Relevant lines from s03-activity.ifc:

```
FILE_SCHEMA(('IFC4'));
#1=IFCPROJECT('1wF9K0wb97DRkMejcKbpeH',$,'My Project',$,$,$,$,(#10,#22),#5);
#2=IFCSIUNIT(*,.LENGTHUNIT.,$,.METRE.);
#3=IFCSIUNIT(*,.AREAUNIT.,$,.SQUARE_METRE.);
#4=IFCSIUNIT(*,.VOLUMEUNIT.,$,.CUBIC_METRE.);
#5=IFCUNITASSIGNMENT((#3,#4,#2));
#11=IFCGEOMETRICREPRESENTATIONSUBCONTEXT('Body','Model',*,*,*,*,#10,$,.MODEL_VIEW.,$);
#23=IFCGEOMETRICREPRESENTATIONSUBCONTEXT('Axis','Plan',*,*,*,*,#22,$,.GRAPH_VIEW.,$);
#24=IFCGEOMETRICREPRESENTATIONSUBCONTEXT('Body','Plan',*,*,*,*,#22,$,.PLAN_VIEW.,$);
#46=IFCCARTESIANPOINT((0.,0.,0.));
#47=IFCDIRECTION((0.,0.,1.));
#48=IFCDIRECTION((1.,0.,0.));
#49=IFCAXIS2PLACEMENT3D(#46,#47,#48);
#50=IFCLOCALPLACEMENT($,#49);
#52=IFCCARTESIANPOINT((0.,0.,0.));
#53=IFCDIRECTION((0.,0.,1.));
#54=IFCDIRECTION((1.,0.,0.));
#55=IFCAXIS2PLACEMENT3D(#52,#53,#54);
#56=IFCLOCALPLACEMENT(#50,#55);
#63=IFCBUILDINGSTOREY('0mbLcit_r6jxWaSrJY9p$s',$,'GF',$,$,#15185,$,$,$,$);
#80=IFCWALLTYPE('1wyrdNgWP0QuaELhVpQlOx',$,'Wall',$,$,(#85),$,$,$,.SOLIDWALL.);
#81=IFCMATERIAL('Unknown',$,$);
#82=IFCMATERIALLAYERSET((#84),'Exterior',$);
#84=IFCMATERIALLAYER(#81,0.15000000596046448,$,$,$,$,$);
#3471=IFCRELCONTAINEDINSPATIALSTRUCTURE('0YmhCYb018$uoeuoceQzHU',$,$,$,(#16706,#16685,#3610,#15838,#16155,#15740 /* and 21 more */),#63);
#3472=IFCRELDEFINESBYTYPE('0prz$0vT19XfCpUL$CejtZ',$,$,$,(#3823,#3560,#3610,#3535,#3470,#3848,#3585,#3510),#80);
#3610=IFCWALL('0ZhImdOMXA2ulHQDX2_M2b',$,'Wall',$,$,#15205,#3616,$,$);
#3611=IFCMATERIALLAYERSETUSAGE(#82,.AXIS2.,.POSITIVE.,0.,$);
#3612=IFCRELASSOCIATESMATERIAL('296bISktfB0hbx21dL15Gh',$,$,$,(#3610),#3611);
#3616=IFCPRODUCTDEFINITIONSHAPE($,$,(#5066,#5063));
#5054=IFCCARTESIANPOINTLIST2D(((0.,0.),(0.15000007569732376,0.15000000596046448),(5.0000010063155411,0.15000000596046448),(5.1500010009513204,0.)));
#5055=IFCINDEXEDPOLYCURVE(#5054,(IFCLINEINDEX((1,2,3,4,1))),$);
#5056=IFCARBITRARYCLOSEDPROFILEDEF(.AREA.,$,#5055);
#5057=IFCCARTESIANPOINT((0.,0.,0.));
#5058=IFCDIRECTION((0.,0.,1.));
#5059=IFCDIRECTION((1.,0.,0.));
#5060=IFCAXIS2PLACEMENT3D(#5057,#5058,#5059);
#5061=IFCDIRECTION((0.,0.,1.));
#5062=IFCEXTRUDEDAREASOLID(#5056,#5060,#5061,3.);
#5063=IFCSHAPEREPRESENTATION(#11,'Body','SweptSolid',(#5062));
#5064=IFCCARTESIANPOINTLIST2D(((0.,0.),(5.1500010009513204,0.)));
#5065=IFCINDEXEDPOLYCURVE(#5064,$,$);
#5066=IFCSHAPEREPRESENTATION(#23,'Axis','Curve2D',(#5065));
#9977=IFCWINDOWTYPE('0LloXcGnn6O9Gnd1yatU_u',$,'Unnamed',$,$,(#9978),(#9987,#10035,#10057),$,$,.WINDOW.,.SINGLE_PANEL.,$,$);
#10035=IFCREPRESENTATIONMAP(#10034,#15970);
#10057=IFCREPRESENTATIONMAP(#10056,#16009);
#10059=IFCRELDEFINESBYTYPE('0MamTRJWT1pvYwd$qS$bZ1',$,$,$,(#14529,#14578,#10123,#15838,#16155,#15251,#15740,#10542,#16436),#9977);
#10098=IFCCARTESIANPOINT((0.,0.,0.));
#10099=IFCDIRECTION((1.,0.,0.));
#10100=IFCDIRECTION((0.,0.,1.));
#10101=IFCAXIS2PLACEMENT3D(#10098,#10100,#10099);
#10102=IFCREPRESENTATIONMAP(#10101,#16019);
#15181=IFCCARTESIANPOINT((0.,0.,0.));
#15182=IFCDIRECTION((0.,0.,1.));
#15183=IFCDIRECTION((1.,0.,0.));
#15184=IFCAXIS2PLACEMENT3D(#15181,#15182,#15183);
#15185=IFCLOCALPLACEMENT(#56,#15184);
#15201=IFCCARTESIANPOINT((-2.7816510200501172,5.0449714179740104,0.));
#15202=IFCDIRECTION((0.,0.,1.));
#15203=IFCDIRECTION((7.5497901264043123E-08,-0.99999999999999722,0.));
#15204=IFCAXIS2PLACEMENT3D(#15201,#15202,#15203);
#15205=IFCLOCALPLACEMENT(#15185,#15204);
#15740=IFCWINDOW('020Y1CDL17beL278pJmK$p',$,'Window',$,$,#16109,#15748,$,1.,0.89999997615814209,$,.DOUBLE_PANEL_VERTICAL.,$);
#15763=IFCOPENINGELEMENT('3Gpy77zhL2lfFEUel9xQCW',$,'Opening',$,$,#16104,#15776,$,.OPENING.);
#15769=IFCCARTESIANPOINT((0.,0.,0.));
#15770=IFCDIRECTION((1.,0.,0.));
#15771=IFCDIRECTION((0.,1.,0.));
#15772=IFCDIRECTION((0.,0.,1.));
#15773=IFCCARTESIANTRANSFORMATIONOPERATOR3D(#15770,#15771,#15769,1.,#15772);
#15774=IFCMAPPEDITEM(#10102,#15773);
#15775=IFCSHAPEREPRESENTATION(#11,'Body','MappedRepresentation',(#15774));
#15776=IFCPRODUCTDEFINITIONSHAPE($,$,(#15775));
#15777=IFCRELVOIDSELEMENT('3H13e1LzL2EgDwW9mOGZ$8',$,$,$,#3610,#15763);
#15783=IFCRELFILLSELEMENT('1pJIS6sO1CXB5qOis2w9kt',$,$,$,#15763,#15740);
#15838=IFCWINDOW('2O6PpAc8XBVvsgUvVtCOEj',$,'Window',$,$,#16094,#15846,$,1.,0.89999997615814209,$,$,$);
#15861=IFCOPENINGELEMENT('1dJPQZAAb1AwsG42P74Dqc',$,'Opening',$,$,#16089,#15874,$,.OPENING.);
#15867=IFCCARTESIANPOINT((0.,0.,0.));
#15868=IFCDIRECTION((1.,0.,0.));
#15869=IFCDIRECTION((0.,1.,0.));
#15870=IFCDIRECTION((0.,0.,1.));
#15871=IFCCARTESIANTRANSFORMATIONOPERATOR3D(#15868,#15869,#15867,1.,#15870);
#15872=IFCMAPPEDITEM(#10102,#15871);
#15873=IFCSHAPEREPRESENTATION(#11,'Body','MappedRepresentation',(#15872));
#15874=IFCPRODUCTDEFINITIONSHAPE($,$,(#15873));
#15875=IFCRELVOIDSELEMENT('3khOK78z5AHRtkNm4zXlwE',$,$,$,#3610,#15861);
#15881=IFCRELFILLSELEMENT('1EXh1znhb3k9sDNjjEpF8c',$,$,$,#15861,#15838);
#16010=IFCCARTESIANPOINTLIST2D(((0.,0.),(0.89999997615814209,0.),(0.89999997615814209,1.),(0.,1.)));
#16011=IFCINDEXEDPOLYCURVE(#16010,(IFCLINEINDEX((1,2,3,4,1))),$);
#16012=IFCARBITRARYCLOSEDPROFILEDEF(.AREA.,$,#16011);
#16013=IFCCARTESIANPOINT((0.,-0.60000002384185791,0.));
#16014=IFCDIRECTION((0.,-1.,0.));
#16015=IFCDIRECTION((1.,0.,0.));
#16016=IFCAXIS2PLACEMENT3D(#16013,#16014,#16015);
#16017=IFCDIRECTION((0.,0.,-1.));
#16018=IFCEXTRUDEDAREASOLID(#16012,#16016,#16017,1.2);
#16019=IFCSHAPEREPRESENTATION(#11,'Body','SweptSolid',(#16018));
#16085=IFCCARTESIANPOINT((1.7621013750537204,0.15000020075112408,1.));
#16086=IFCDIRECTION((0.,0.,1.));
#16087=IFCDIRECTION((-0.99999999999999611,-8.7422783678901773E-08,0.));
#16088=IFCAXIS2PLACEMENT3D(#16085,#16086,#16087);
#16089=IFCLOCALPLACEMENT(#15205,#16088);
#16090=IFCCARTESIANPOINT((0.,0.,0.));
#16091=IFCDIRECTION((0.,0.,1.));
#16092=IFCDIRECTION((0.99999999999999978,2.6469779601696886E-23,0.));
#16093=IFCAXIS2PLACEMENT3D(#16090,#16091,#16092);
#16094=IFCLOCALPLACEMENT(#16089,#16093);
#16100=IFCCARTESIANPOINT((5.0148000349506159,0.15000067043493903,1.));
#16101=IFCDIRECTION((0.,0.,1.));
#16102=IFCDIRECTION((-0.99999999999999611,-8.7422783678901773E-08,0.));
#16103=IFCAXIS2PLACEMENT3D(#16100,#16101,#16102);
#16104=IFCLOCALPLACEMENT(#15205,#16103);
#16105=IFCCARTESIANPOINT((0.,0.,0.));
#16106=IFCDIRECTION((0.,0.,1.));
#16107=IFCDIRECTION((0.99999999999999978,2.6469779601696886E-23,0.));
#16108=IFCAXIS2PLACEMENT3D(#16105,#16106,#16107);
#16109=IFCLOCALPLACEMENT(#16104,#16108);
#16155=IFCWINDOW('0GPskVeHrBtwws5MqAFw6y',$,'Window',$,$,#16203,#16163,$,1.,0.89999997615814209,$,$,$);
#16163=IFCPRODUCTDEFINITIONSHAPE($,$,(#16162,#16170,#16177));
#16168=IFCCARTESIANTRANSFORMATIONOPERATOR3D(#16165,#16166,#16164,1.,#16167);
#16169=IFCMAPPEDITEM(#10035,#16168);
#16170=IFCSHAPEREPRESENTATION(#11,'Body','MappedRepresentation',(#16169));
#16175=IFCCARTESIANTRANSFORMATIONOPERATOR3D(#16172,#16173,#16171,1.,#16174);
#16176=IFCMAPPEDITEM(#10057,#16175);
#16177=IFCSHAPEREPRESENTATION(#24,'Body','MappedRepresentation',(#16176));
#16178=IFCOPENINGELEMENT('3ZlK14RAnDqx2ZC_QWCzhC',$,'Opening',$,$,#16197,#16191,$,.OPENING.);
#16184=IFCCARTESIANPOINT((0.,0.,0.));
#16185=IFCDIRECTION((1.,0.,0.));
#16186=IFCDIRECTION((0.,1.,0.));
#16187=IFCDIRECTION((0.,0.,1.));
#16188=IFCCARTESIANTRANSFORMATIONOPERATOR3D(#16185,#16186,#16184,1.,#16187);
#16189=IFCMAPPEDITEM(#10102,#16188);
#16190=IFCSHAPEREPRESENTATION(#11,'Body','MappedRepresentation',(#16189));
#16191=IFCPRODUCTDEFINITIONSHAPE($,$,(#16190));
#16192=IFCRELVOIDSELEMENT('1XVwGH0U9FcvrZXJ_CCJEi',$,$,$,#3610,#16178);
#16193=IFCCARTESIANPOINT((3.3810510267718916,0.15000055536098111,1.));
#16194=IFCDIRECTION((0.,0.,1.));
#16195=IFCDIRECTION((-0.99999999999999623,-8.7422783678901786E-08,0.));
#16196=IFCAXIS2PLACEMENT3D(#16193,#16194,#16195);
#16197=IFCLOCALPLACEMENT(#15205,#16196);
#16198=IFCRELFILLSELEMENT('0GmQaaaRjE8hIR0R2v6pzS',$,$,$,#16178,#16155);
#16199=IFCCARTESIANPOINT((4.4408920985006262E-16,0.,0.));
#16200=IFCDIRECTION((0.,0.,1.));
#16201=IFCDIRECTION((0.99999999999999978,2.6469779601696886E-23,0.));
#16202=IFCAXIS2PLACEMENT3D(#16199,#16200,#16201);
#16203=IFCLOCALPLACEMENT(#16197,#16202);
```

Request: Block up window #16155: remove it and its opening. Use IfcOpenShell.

```python
import ifcopenshell
import ifcopenshell.api.feature
import ifcopenshell.api.root
import ifcopenshell.geom
import ifcopenshell.util.shape

model = ifcopenshell.open("s03-activity.ifc")
settings = ifcopenshell.geom.settings()


def volume(element):
    """Net volume in cubic metres, openings subtracted."""
    shape = ifcopenshell.geom.create_shape(settings, element)
    return ifcopenshell.util.shape.get_volume(shape.geometry)


window = model.by_guid("0GPskVeHrBtwws5MqAFw6y")
opening = window.FillsVoids[0].RelatingOpeningElement
wall = opening.VoidsElements[0].RelatingBuildingElement
before = volume(wall)

ifcopenshell.api.root.remove_product(model, product=window)
ifcopenshell.api.feature.remove_feature(model, feature=opening)

after = volume(wall)

print(f"wall volume {before:.3f} -> {after:.3f} m3")

model.write("s03-activity_edited.ifc")
```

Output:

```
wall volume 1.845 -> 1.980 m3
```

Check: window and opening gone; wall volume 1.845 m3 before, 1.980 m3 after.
